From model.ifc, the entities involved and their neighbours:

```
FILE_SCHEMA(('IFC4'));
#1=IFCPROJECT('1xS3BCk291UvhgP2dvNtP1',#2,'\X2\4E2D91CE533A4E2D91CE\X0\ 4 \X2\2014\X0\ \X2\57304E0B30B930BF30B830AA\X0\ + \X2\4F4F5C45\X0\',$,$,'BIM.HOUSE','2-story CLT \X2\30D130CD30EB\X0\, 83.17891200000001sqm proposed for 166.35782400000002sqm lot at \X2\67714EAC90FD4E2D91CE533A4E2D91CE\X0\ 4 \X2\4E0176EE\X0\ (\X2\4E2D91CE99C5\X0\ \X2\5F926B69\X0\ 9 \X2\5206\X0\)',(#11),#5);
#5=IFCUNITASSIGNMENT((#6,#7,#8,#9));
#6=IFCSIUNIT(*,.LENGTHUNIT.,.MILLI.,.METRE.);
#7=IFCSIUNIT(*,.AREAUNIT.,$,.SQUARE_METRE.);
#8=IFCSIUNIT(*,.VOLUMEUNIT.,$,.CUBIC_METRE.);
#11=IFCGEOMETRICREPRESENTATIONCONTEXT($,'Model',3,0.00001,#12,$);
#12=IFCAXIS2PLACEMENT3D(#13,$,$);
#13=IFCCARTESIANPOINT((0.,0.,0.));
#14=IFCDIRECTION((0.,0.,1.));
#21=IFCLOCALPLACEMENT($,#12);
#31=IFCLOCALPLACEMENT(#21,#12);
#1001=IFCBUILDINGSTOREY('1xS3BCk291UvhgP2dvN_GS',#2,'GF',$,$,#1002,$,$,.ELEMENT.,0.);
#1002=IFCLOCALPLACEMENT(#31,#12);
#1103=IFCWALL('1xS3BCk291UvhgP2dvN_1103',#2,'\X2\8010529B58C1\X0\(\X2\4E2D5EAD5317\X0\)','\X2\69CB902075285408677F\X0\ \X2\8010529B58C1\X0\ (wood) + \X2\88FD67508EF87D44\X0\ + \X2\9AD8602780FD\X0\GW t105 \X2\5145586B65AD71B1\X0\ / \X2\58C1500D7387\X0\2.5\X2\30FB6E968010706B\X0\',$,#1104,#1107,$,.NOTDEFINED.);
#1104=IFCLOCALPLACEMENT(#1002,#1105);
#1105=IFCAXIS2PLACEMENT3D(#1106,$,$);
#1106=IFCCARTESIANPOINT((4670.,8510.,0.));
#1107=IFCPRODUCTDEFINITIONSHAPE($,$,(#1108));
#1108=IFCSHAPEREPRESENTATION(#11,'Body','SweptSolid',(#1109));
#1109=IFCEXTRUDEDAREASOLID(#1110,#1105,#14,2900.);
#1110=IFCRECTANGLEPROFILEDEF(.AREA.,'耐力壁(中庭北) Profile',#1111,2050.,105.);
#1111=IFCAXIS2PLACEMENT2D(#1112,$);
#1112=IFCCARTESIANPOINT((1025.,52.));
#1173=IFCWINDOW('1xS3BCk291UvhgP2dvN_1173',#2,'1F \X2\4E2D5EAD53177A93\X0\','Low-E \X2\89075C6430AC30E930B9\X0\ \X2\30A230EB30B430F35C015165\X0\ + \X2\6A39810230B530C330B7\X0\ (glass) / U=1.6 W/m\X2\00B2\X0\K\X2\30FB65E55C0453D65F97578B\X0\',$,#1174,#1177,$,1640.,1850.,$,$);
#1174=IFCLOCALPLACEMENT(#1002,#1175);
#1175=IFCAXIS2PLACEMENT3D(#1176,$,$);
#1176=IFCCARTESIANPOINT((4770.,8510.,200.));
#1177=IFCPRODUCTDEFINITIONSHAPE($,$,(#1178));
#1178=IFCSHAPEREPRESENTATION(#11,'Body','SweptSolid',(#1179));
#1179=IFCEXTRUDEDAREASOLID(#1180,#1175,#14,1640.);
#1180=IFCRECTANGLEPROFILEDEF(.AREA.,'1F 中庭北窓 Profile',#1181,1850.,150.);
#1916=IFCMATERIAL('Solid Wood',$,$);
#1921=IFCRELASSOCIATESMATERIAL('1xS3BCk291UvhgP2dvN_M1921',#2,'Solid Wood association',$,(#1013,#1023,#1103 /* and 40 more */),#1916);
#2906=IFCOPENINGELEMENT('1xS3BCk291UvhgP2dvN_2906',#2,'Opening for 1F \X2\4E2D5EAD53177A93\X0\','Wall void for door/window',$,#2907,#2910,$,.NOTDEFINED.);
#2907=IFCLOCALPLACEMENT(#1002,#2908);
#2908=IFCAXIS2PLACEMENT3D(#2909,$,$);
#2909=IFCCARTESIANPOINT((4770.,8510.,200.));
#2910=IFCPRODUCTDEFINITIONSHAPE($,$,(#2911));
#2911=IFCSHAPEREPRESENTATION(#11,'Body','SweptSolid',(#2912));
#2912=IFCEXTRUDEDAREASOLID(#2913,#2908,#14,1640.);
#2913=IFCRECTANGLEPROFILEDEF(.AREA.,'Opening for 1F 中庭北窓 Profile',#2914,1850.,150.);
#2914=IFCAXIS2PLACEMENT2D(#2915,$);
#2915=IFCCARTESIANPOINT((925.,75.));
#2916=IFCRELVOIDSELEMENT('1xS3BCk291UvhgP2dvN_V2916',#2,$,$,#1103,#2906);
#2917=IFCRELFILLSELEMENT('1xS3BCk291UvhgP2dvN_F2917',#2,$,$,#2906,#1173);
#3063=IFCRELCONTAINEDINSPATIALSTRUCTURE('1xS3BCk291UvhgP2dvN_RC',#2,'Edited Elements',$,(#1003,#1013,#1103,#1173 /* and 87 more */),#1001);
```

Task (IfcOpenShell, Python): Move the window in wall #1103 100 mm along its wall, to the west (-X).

```python
import ifcopenshell
import ifcopenshell.api.geometry
import ifcopenshell.util.placement
import ifcopenshell.util.unit

model = ifcopenshell.open("model.ifc")
unit_scale = ifcopenshell.util.unit.calculate_unit_scale(model)

window = model.by_guid("1xS3BCk291UvhgP2dvN_1173")
opening = window.FillsVoids[0].RelatingOpeningElement
wall = opening.VoidsElements[0].RelatingBuildingElement

wall_matrix = ifcopenshell.util.placement.get_local_placement(wall.ObjectPlacement)
shift = wall_matrix[:3, 0] * -0.1 / unit_scale
before = ifcopenshell.util.placement.get_local_placement(window.ObjectPlacement)[:3, 3].copy()

# The window is not placed relative to its opening, so move both.
for product in (opening, window):
    matrix = ifcopenshell.util.placement.get_local_placement(product.ObjectPlacement)
    matrix[:3, 3] += shift
    ifcopenshell.api.geometry.edit_object_placement(model, product=product, matrix=matrix, is_si=False)

after = ifcopenshell.util.placement.get_local_placement(window.ObjectPlacement)[:3, 3]
print("window moved by", (after - before).round(3) + 0.0)

model.write("model-out.ifc")
```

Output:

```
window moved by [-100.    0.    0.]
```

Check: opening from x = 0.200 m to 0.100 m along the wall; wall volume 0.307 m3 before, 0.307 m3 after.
